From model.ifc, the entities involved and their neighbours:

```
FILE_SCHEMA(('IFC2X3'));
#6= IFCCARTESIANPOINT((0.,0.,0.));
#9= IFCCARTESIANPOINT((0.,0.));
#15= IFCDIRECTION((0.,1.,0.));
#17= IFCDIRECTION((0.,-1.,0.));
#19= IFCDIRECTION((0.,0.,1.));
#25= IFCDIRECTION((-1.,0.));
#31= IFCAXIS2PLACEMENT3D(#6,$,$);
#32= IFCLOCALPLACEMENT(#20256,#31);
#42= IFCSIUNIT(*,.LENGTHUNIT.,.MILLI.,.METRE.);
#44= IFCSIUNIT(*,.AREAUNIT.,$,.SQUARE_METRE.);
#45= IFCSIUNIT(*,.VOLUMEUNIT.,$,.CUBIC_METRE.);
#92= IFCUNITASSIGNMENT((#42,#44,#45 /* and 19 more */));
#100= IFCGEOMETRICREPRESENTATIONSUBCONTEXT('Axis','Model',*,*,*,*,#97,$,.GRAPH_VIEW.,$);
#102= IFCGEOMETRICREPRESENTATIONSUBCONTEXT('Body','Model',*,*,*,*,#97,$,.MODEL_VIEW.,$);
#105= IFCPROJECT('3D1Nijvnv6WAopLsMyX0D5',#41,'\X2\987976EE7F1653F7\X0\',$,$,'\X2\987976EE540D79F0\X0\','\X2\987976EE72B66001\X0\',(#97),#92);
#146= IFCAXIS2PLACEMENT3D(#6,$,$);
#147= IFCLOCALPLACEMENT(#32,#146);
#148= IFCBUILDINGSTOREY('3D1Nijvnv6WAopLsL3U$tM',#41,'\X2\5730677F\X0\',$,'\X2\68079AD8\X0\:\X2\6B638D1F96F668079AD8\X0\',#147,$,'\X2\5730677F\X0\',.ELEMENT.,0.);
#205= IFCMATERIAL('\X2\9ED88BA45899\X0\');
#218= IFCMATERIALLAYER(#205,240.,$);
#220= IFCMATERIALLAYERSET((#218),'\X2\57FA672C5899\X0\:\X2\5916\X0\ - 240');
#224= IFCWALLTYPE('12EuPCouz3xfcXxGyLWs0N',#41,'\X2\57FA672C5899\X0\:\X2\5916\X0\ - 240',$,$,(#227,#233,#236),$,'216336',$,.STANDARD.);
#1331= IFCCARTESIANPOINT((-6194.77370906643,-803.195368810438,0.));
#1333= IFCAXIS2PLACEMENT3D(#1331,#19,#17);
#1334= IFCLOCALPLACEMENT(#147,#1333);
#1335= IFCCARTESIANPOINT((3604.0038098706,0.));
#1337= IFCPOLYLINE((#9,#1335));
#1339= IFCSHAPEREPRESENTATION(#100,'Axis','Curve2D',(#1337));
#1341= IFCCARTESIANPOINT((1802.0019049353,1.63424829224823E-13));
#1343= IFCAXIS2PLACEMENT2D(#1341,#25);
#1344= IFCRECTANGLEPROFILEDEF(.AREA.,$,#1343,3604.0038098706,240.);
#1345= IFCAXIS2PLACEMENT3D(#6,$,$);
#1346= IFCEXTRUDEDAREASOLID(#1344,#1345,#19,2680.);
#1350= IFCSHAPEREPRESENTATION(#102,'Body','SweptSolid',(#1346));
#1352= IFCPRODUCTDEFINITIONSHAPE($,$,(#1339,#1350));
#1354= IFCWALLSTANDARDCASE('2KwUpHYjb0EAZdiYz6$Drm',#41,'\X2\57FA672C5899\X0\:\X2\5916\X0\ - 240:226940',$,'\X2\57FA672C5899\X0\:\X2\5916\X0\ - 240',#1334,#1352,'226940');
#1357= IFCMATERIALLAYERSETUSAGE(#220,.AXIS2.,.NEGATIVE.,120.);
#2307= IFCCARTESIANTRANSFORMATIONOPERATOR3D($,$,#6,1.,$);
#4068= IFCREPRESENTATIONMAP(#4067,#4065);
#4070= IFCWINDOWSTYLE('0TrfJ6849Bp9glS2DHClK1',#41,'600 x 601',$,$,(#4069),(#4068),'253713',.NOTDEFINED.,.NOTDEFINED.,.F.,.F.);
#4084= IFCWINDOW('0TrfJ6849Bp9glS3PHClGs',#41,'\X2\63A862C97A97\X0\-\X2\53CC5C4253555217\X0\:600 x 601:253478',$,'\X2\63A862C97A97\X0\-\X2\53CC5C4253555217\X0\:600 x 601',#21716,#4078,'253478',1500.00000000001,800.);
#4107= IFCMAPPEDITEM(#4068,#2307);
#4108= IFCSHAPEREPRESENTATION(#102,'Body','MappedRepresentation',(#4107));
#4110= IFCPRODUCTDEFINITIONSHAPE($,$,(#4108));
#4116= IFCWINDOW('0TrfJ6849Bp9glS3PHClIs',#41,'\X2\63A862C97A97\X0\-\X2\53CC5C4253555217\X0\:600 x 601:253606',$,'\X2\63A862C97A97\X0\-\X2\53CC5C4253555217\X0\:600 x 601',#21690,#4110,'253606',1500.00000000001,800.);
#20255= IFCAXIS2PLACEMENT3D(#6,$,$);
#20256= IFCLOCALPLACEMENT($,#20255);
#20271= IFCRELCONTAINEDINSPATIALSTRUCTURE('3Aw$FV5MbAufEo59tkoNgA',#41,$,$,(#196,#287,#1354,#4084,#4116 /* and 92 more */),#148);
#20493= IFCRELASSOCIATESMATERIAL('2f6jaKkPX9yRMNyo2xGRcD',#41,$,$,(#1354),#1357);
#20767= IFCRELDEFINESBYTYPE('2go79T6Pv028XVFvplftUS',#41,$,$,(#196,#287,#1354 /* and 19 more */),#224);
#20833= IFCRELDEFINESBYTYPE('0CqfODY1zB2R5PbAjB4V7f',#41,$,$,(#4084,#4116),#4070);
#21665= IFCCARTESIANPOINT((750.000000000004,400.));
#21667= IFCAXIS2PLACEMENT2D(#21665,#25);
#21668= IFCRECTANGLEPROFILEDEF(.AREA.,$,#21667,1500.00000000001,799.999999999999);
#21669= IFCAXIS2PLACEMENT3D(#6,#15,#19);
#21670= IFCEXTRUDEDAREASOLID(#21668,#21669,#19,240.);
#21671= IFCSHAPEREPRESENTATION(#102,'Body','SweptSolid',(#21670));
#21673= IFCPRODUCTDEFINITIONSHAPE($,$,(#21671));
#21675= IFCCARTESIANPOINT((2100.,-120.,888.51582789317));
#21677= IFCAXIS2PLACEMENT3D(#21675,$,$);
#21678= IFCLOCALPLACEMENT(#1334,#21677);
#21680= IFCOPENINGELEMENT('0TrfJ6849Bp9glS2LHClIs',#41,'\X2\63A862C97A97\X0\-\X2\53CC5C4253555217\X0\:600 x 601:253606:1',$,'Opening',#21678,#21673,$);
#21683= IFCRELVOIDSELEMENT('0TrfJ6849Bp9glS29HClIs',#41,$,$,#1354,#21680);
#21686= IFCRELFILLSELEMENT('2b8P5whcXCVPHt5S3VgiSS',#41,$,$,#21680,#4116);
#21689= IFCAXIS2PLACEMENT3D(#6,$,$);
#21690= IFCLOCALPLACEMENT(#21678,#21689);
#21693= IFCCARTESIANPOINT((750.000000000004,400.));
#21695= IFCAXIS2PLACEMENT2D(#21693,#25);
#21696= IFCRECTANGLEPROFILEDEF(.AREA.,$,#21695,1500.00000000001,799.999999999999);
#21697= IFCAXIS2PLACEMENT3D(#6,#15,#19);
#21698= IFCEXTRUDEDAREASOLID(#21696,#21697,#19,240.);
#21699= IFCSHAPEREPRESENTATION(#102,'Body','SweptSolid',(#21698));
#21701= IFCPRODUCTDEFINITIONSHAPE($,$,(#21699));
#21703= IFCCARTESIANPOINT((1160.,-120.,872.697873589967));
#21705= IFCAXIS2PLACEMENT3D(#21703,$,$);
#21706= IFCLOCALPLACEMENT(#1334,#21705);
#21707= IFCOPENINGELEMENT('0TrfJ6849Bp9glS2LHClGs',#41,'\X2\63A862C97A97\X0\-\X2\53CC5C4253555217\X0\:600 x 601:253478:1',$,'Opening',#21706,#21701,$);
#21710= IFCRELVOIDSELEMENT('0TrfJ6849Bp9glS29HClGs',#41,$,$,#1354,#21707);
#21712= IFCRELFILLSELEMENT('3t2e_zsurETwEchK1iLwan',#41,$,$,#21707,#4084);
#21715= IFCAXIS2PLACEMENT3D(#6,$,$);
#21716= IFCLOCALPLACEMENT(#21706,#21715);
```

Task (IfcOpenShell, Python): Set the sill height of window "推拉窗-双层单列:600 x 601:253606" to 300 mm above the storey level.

```python
import numpy as np
import ifcopenshell
import ifcopenshell.api.geometry
import ifcopenshell.geom
import ifcopenshell.util.element
import ifcopenshell.util.placement
import ifcopenshell.util.shape
import ifcopenshell.util.unit

model = ifcopenshell.open("model.ifc")
unit_scale = ifcopenshell.util.unit.calculate_unit_scale(model)

window = model.by_guid("0TrfJ6849Bp9glS3PHClIs")
opening = window.FillsVoids[0].RelatingOpeningElement
storey = ifcopenshell.util.element.get_container(window, ifc_class="IfcBuildingStorey")
level = ifcopenshell.util.placement.get_local_placement(storey.ObjectPlacement)[2, 3]

# The opening's origin need not be at the sill, so measure its lowest point.
shape = ifcopenshell.geom.create_shape(ifcopenshell.geom.settings(), opening)
bottom = ifcopenshell.util.shape.get_shape_bottom_elevation(shape, shape.geometry) / unit_scale
dz = level + 0.3 / unit_scale - bottom

shift = np.array([0.0, 0.0, dz])
# The window is placed relative to its opening, so it follows when the opening moves.
matrix = ifcopenshell.util.placement.get_local_placement(opening.ObjectPlacement)
matrix[:3, 3] += shift
ifcopenshell.api.geometry.edit_object_placement(
    model, product=opening, matrix=matrix, is_si=False, should_transform_children=True
)

print(f"moved by {dz * unit_scale:+.3f} m")

model.write("model-out.ifc")
```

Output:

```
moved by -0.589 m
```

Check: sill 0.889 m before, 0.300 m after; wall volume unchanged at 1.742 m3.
